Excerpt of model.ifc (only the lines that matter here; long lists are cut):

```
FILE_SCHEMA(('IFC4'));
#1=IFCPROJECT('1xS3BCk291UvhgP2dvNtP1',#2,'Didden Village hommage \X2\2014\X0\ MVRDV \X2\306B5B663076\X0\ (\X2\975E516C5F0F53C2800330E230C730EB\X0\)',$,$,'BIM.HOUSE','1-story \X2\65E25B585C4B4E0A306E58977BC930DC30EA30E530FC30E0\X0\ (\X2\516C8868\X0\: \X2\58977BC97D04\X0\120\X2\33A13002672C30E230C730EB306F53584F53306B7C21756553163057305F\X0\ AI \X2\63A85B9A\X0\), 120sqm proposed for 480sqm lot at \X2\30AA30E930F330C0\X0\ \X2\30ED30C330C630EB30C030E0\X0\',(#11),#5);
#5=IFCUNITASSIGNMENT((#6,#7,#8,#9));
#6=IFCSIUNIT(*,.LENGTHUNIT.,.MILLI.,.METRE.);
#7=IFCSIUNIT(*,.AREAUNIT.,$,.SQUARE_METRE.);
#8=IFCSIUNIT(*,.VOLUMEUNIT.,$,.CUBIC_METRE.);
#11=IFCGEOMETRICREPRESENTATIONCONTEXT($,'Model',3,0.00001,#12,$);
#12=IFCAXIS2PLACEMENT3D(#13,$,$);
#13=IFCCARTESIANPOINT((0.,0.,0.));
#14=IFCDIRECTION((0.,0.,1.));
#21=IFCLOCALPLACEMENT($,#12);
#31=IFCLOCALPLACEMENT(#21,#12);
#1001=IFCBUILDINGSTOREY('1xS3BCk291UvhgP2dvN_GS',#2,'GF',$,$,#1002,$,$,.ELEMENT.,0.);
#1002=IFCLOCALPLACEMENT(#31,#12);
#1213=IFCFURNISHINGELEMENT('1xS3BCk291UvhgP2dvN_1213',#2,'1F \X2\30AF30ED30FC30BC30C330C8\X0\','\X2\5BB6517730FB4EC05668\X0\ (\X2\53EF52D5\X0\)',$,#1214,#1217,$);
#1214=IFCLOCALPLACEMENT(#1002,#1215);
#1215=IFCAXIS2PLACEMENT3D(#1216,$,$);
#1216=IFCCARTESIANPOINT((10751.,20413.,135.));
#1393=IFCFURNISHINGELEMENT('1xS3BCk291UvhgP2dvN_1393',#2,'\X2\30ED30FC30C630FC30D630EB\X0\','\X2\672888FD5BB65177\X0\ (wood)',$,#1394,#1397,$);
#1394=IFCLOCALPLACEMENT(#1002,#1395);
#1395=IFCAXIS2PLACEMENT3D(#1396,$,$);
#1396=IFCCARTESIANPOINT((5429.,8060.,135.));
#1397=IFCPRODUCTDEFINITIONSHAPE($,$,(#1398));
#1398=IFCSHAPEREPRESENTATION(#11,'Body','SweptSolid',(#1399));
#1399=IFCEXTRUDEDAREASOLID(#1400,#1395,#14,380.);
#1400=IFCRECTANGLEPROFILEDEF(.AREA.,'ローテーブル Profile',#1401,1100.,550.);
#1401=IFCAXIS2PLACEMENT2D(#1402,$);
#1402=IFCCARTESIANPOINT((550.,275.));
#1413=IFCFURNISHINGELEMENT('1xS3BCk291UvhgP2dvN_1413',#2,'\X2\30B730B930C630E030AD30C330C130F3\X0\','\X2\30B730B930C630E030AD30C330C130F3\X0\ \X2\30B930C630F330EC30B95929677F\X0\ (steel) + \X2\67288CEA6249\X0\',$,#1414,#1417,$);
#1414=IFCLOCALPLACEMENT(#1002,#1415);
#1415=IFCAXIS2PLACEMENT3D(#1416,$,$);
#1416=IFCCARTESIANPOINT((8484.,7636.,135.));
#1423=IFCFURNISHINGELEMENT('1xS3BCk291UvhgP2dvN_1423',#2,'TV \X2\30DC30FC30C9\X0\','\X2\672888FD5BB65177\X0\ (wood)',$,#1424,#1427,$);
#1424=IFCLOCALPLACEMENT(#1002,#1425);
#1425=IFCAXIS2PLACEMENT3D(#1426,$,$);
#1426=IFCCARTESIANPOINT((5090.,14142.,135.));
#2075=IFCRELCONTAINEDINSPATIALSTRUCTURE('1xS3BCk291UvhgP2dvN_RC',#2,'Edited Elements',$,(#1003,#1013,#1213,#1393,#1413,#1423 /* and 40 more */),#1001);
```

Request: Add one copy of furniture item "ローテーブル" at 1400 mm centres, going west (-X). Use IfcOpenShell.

```python
import numpy as np
import ifcopenshell
import ifcopenshell.api.geometry
import ifcopenshell.api.root
import ifcopenshell.util.element
import ifcopenshell.util.placement
import ifcopenshell.util.unit

model = ifcopenshell.open("model.ifc")
unit_scale = ifcopenshell.util.unit.calculate_unit_scale(model)


def reuse_history(source, copy):
    """copy_class also copies each property set's owner history, people and application; keep the originals."""
    for rel in copy.IsDefinedBy:
        if rel.is_a("IfcRelDefinesByProperties") and (history := rel.RelatingPropertyDefinition.OwnerHistory):
            rel.RelatingPropertyDefinition.OwnerHistory = source.OwnerHistory
            ifcopenshell.util.element.remove_deep2(model, history)


source = model.by_id(1393)
base = ifcopenshell.util.placement.get_local_placement(source.ObjectPlacement)
step = np.array([-1.0, 0.0, 0.0]) * 1.4 / unit_scale

for i in range(1, 2):
    copy = ifcopenshell.api.root.copy_class(model, product=source)
    copy.Representation = ifcopenshell.util.element.copy_deep(
        model, source.Representation, exclude=["IfcGeometricRepresentationContext", "IfcRepresentationMap"]
    )
    reuse_history(source, copy)
    matrix = base.copy()
    matrix[:3, 3] += i * step
    print("added at", matrix[:3, 3].round(3) + 0.0)
    ifcopenshell.api.geometry.edit_object_placement(model, product=copy, matrix=matrix, is_si=False)

model.write("model_edited.ifc")
```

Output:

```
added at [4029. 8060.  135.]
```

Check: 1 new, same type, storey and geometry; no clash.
